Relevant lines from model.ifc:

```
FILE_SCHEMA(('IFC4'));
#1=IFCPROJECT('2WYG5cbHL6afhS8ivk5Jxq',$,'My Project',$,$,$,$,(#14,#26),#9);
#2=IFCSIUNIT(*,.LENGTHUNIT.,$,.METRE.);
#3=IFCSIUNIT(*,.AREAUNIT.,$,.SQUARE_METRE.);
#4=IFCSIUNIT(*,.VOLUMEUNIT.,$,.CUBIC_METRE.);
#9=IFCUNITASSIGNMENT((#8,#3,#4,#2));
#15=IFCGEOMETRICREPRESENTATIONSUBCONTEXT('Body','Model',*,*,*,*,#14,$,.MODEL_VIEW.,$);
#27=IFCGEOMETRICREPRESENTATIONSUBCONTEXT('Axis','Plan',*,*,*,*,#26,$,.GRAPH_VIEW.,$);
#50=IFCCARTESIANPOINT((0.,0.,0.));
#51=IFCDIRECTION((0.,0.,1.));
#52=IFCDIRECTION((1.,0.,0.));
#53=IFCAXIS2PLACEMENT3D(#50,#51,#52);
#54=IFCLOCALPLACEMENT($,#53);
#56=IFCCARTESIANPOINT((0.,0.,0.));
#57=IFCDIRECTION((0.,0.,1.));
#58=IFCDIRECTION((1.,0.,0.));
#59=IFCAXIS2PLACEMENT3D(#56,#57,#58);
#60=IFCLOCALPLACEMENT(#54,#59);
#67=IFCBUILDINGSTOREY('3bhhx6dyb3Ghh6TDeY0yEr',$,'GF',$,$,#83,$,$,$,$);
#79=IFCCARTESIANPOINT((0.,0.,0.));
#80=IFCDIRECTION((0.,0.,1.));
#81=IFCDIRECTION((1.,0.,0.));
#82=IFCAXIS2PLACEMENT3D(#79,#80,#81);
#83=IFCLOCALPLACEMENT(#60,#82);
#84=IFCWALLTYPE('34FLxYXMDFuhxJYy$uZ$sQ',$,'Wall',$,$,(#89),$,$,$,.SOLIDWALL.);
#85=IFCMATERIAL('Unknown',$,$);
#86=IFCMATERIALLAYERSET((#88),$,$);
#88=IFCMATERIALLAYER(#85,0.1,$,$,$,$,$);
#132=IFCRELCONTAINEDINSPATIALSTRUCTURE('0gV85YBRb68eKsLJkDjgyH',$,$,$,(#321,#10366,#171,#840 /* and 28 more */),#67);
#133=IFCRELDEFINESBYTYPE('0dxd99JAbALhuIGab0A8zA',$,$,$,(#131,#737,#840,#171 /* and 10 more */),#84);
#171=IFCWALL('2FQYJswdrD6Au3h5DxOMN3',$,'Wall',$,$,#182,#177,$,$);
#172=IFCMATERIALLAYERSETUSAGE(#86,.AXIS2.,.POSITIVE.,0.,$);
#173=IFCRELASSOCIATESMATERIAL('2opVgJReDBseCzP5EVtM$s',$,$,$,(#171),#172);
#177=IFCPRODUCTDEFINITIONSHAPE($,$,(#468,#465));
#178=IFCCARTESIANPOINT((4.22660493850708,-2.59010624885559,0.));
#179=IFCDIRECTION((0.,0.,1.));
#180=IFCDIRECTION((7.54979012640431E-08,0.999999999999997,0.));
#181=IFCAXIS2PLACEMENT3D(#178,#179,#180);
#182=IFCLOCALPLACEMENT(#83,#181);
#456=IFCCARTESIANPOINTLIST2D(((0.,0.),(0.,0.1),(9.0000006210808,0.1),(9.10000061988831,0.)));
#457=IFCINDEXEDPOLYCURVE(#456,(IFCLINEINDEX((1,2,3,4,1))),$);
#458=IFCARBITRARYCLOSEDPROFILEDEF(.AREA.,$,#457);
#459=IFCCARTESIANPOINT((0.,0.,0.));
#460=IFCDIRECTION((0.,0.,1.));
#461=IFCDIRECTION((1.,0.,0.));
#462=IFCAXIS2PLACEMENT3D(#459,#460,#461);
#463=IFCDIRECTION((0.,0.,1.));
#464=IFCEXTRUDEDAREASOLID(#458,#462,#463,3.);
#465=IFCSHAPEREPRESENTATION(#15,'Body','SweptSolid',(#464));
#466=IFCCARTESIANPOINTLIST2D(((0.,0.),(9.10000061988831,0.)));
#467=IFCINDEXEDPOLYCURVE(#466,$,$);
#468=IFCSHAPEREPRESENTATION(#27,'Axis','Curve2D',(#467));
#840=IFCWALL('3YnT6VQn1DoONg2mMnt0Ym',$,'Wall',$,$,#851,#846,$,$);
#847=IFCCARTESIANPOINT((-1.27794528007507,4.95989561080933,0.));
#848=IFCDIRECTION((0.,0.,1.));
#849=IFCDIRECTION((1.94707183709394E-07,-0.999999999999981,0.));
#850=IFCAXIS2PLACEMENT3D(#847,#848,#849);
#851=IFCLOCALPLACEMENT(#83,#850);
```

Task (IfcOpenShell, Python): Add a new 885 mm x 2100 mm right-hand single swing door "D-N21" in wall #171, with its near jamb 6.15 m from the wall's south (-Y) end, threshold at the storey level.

```python
import numpy as np
import ifcopenshell
import ifcopenshell.api.feature
import ifcopenshell.api.geometry
import ifcopenshell.api.root
import ifcopenshell.api.spatial
import ifcopenshell.geom
import ifcopenshell.util.element
import ifcopenshell.util.placement
import ifcopenshell.util.representation
import ifcopenshell.util.shape
import ifcopenshell.util.unit

model = ifcopenshell.open("model.ifc")
unit_scale = ifcopenshell.util.unit.calculate_unit_scale(model)
settings = ifcopenshell.geom.settings()


def volume(element):
    """Net volume in cubic metres, openings subtracted."""
    shape = ifcopenshell.geom.create_shape(settings, element)
    return ifcopenshell.util.shape.get_volume(shape.geometry)


wall = model.by_guid("2FQYJswdrD6Au3h5DxOMN3")
storey = ifcopenshell.util.element.get_container(wall, ifc_class="IfcBuildingStorey")
context = ifcopenshell.util.representation.get_context(model, "Model", "Body", "MODEL_VIEW")
before = volume(wall)

width, height, from_end, sill = 0.885, 2.1, 6.15, 0.0  # metres

# The wall runs along its own X axis, and the end named is its -X end.
wall_shape = ifcopenshell.geom.create_shape(settings, wall)
x, y, z = ifcopenshell.util.shape.get_vertices(wall_shape.geometry).T
start = x.min() + from_end
face, thickness = float(y.min()), float(y.max() - y.min())
wall_matrix = ifcopenshell.util.placement.get_local_placement(wall.ObjectPlacement)
level = ifcopenshell.util.placement.get_local_placement(storey.ObjectPlacement)[2, 3]


def in_wall(x, y):
    """Placement at x, y metres in the wall's axes, at sill height."""
    matrix = wall_matrix.copy()
    matrix[:, 3] = wall_matrix @ np.array([x / unit_scale, y / unit_scale, 0.0, 1.0])
    matrix[2, 3] = level + sill / unit_scale
    return matrix


# Opening: a box that overshoots both wall faces by 50 mm.
opening = ifcopenshell.api.root.create_entity(model, ifc_class="IfcOpeningElement", predefined_type="OPENING")
box = ifcopenshell.api.geometry.add_wall_representation(
    model, context=context, length=width, height=height, thickness=thickness + 0.1
)
ifcopenshell.api.geometry.assign_representation(model, product=opening, representation=box)
ifcopenshell.api.geometry.edit_object_placement(model, product=opening, matrix=in_wall(start, face - 0.05), is_si=False)
ifcopenshell.api.feature.add_feature(model, feature=opening, element=wall)

door = ifcopenshell.api.root.create_entity(model, ifc_class="IfcDoor", name="D-N21", predefined_type="DOOR")
door.OverallWidth, door.OverallHeight = width / unit_scale, height / unit_scale
door.OperationType = "SINGLE_SWING_RIGHT"
body = ifcopenshell.api.geometry.add_door_representation(
    model,
    context=context,
    overall_width=door.OverallWidth,
    overall_height=door.OverallHeight,
    operation_type="SINGLE_SWING_RIGHT",
    lining_properties={"LiningDepth": thickness / unit_scale, "ThresholdDepth": thickness / unit_scale},
)
ifcopenshell.api.geometry.assign_representation(model, product=door, representation=body)
ifcopenshell.api.spatial.assign_container(model, products=[door], relating_structure=storey)
ifcopenshell.api.feature.add_filling(model, opening=opening, element=door)

# The lining spans the wall, so the door starts at the wall face.
ifcopenshell.api.geometry.edit_object_placement(model, product=door, matrix=in_wall(start, face), is_si=False)

after = volume(wall)

print(f"wall volume {before:.3f} -> {after:.3f} m3")

model.write("model_updated.ifc")
```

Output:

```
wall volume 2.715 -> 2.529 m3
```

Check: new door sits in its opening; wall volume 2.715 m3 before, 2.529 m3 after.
